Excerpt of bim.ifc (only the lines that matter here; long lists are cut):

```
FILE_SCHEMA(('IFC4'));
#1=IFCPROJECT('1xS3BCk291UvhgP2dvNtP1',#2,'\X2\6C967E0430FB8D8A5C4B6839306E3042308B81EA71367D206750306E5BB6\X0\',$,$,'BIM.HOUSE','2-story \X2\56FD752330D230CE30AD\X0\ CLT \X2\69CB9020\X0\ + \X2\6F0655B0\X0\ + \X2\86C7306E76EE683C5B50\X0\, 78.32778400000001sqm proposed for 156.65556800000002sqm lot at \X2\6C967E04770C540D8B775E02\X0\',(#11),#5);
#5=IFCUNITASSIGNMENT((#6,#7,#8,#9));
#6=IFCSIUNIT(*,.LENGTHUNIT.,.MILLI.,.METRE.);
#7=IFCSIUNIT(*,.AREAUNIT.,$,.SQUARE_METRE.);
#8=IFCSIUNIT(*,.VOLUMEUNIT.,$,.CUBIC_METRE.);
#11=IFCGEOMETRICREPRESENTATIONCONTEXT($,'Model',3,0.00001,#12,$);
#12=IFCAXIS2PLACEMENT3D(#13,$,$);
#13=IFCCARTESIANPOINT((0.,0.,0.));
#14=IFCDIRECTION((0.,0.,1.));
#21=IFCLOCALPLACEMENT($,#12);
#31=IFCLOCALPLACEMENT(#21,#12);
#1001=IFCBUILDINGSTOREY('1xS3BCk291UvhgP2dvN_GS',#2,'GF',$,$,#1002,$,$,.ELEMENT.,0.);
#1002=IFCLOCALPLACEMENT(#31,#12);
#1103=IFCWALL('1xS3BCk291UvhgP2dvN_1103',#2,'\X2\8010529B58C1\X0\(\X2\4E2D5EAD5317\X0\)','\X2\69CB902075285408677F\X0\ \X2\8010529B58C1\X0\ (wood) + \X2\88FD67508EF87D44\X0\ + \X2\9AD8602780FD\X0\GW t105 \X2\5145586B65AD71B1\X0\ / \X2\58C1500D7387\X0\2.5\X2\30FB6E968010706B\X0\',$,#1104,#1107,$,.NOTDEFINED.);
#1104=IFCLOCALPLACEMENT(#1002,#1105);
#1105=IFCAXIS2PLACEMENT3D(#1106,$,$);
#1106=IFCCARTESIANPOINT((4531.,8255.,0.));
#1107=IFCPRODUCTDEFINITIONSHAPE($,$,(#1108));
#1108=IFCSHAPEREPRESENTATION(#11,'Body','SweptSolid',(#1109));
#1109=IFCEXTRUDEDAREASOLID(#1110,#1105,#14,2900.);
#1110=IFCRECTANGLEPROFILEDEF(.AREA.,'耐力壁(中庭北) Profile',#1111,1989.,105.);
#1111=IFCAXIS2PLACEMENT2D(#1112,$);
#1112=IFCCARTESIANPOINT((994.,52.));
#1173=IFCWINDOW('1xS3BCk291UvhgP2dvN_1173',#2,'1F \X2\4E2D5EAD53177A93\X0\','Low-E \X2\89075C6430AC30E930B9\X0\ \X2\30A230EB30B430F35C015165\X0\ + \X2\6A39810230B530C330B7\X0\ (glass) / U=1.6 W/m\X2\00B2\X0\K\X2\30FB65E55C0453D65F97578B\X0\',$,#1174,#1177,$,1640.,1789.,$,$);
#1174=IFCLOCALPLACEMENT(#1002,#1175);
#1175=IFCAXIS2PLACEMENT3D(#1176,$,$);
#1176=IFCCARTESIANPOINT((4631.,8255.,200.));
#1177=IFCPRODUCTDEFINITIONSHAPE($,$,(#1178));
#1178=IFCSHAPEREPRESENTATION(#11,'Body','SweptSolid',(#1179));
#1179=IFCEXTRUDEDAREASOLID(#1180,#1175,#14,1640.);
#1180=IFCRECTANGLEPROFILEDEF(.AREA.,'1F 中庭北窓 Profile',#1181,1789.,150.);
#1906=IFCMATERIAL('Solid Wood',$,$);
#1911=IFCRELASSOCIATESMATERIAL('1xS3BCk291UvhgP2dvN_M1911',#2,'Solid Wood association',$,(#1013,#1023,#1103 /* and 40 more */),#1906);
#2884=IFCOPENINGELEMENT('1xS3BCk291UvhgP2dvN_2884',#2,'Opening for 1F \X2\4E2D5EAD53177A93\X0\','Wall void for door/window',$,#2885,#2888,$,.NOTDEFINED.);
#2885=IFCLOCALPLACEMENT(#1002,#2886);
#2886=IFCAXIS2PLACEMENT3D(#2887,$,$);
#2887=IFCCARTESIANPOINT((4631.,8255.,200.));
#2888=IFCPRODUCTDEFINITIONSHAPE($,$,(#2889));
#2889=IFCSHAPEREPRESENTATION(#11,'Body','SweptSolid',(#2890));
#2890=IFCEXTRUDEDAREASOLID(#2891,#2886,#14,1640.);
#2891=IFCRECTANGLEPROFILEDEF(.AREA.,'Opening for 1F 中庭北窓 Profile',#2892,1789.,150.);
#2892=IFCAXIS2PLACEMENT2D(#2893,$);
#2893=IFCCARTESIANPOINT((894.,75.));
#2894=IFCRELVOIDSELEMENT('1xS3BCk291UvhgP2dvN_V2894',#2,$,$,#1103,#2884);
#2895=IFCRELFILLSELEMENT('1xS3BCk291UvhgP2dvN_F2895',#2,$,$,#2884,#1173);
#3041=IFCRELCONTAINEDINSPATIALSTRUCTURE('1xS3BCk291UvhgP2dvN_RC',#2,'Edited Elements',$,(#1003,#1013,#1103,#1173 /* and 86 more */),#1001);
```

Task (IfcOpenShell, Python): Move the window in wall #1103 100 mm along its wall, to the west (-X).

```python
import ifcopenshell
import ifcopenshell.api.geometry
import ifcopenshell.util.placement
import ifcopenshell.util.unit

model = ifcopenshell.open("bim.ifc")
unit_scale = ifcopenshell.util.unit.calculate_unit_scale(model)

window = model.by_id(1173)
opening = window.FillsVoids[0].RelatingOpeningElement
wall = opening.VoidsElements[0].RelatingBuildingElement

wall_matrix = ifcopenshell.util.placement.get_local_placement(wall.ObjectPlacement)
shift = wall_matrix[:3, 0] * -0.1 / unit_scale
before = ifcopenshell.util.placement.get_local_placement(window.ObjectPlacement)[:3, 3].copy()

# The window is not placed relative to its opening, so move both.
for product in (opening, window):
    matrix = ifcopenshell.util.placement.get_local_placement(product.ObjectPlacement)
    matrix[:3, 3] += shift
    ifcopenshell.api.geometry.edit_object_placement(model, product=product, matrix=matrix, is_si=False)

after = ifcopenshell.util.placement.get_local_placement(window.ObjectPlacement)[:3, 3]
print("window moved by", (after - before).round(3) + 0.0)

model.write("bim_edited.ifc")
```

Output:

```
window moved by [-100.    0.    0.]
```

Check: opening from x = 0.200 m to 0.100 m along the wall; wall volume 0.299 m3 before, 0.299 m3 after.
